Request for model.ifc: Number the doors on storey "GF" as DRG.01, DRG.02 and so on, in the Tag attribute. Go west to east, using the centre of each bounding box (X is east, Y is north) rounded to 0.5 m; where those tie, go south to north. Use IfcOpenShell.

First a look at what the model holds.

```python
import ifcopenshell
import ifcopenshell.util.element
import ifcopenshell.util.placement

model = ifcopenshell.open("model.ifc")
print(model.schema)
storey = next(s for s in model.by_type("IfcBuildingStorey") if s.Name == "GF")
doors = [e for e in ifcopenshell.util.element.get_decomposition(storey) if e.is_a("IfcDoor")]
for e in sorted(doors, key=lambda e: e.id()):
    origin = ifcopenshell.util.placement.get_local_placement(e.ObjectPlacement)[:3, 3]
    print(e.id(), e.Tag, e.Name, origin.round(2) + 0.0, sep=" | ")
```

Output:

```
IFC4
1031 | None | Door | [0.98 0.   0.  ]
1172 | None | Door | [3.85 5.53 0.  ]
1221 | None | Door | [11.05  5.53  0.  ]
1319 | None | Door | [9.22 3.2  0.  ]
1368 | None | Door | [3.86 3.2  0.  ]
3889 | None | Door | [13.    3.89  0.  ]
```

```python
import ifcopenshell
import ifcopenshell.geom
import ifcopenshell.util.element
import ifcopenshell.util.shape

model = ifcopenshell.open("model.ifc")
settings = ifcopenshell.geom.settings()
settings.set("use-world-coords", True)


def centre(element):
    shape = ifcopenshell.geom.create_shape(settings, element)
    return ifcopenshell.util.shape.get_bbox_centroid(shape.geometry)


storey = next(s for s in model.by_type("IfcBuildingStorey") if s.Name == "GF")
doors = [e for e in ifcopenshell.util.element.get_decomposition(storey) if e.is_a("IfcDoor")]

# Insertion points can sit at a corner or the storey origin, so sort by the geometry (in metres).
centres = {e: centre(e) for e in doors}
doors.sort(key=lambda e: (round(centres[e][0] / 0.5), centres[e][1]))

for i, e in enumerate(doors, start=1):
    number = f"DRG.{i:02d}"
    e.Tag = number
    print(e.id(), number)

model.write("model_rev.ifc")
```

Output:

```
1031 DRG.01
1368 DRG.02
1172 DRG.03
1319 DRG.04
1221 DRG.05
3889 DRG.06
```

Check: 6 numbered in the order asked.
